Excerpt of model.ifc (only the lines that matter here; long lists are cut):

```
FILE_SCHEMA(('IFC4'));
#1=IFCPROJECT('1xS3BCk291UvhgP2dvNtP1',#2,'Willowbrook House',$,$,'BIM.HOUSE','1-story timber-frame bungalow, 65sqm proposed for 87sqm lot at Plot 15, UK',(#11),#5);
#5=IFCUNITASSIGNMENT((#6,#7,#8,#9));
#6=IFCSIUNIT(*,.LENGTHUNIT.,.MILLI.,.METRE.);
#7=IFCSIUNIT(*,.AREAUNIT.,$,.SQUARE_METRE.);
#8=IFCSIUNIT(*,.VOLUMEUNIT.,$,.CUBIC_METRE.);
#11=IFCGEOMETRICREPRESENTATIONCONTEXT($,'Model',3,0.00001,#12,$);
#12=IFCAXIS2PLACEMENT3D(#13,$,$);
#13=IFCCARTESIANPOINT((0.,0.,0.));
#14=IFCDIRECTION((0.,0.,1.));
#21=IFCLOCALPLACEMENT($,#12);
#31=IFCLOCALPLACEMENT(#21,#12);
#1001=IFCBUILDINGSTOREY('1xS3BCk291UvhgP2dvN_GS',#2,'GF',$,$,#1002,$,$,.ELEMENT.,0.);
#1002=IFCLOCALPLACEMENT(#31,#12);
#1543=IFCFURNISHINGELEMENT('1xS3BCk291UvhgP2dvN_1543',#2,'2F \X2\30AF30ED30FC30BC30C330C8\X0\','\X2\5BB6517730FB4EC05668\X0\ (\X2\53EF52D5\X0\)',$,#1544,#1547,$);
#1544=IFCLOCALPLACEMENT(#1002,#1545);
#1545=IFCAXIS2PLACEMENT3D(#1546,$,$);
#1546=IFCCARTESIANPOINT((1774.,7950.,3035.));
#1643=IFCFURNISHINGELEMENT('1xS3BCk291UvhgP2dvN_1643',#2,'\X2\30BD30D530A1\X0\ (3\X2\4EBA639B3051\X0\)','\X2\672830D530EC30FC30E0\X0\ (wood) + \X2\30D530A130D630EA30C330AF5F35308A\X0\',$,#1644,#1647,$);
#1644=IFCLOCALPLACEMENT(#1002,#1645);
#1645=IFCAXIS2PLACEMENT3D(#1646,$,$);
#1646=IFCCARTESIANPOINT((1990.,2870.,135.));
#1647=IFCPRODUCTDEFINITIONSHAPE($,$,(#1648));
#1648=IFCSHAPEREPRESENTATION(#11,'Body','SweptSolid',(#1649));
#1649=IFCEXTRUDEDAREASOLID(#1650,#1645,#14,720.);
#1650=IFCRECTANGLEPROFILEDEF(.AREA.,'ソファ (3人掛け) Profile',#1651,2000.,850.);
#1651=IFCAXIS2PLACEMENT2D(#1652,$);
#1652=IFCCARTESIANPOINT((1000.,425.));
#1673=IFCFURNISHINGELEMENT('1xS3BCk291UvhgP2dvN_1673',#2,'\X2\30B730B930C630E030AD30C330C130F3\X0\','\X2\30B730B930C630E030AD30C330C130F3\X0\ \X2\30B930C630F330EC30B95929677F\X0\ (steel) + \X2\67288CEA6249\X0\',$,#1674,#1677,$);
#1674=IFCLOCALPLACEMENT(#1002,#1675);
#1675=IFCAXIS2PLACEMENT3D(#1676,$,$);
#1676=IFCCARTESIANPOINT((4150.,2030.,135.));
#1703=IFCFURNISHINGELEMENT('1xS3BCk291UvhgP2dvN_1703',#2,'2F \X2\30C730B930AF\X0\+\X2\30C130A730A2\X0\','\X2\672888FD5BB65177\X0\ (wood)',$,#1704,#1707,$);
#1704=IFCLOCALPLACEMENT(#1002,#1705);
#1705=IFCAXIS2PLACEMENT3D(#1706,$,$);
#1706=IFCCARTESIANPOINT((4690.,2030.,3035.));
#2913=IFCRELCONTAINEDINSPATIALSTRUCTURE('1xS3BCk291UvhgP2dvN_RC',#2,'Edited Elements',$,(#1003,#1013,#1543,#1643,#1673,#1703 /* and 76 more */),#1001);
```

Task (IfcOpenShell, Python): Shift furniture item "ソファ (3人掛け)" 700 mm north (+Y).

```python
import ifcopenshell
import ifcopenshell.api.geometry
import ifcopenshell.util.placement
import ifcopenshell.util.unit

model = ifcopenshell.open("model.ifc")
unit_scale = ifcopenshell.util.unit.calculate_unit_scale(model)

item = model.by_id(1643)
matrix = ifcopenshell.util.placement.get_local_placement(item.ObjectPlacement)
matrix[1, 3] += 0.7 / unit_scale
ifcopenshell.api.geometry.edit_object_placement(model, product=item, matrix=matrix, is_si=False)

print(ifcopenshell.util.placement.get_local_placement(item.ObjectPlacement).round(3) + 0.0)

model.write("model-out.ifc")
```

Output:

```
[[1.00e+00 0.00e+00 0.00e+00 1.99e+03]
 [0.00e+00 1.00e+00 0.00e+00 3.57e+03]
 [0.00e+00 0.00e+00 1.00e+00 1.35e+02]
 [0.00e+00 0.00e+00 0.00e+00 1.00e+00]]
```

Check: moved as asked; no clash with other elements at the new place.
